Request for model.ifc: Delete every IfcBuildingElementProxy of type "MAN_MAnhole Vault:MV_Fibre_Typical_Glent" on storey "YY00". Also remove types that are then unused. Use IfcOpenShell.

First a look at what the model holds.

```python
import ifcopenshell
import ifcopenshell.util.element

model = ifcopenshell.open("model.ifc")
print(model.schema)
storey = next(s for s in model.by_type("IfcBuildingStorey") if s.Name == "YY00")
proxies = [e for e in ifcopenshell.util.element.get_decomposition(storey) if e.is_a("IfcBuildingElementProxy")]
seen = {}
for e in proxies:
    element_type = ifcopenshell.util.element.get_type(e)
    name = element_type.Name if element_type not in (None, e) else None
    seen[name] = seen.get(name, 0) + 1
for name, count in sorted(seen.items(), key=str):
    print(count, "x", name)
```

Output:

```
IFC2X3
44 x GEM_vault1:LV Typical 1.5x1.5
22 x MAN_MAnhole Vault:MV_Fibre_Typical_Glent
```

```python
import ifcopenshell
import ifcopenshell.api.root
import ifcopenshell.util.element

model = ifcopenshell.open("model.ifc")

storey = next(s for s in model.by_type("IfcBuildingStorey") if s.Name == "YY00")
proxies = [e for e in ifcopenshell.util.element.get_decomposition(storey) if e.is_a("IfcBuildingElementProxy")]
targets = [e for e in proxies if (t := ifcopenshell.util.element.get_type(e)) not in (None, e) and t.Name == "MAN_MAnhole Vault:MV_Fibre_Typical_Glent"]
types = {ifcopenshell.util.element.get_type(e) for e in targets} - {None, *targets}

for e in targets:
    ifcopenshell.api.root.remove_product(model, product=e)
print(len(targets), "removed")

unused = [t for t in types if not ifcopenshell.util.element.get_types(t)]
for t in unused:
    ifcopenshell.api.root.remove_product(model, product=t)
print(len(unused), "unused types removed")

model.write("model_v2.ifc")
```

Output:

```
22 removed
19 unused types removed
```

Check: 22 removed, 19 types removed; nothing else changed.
